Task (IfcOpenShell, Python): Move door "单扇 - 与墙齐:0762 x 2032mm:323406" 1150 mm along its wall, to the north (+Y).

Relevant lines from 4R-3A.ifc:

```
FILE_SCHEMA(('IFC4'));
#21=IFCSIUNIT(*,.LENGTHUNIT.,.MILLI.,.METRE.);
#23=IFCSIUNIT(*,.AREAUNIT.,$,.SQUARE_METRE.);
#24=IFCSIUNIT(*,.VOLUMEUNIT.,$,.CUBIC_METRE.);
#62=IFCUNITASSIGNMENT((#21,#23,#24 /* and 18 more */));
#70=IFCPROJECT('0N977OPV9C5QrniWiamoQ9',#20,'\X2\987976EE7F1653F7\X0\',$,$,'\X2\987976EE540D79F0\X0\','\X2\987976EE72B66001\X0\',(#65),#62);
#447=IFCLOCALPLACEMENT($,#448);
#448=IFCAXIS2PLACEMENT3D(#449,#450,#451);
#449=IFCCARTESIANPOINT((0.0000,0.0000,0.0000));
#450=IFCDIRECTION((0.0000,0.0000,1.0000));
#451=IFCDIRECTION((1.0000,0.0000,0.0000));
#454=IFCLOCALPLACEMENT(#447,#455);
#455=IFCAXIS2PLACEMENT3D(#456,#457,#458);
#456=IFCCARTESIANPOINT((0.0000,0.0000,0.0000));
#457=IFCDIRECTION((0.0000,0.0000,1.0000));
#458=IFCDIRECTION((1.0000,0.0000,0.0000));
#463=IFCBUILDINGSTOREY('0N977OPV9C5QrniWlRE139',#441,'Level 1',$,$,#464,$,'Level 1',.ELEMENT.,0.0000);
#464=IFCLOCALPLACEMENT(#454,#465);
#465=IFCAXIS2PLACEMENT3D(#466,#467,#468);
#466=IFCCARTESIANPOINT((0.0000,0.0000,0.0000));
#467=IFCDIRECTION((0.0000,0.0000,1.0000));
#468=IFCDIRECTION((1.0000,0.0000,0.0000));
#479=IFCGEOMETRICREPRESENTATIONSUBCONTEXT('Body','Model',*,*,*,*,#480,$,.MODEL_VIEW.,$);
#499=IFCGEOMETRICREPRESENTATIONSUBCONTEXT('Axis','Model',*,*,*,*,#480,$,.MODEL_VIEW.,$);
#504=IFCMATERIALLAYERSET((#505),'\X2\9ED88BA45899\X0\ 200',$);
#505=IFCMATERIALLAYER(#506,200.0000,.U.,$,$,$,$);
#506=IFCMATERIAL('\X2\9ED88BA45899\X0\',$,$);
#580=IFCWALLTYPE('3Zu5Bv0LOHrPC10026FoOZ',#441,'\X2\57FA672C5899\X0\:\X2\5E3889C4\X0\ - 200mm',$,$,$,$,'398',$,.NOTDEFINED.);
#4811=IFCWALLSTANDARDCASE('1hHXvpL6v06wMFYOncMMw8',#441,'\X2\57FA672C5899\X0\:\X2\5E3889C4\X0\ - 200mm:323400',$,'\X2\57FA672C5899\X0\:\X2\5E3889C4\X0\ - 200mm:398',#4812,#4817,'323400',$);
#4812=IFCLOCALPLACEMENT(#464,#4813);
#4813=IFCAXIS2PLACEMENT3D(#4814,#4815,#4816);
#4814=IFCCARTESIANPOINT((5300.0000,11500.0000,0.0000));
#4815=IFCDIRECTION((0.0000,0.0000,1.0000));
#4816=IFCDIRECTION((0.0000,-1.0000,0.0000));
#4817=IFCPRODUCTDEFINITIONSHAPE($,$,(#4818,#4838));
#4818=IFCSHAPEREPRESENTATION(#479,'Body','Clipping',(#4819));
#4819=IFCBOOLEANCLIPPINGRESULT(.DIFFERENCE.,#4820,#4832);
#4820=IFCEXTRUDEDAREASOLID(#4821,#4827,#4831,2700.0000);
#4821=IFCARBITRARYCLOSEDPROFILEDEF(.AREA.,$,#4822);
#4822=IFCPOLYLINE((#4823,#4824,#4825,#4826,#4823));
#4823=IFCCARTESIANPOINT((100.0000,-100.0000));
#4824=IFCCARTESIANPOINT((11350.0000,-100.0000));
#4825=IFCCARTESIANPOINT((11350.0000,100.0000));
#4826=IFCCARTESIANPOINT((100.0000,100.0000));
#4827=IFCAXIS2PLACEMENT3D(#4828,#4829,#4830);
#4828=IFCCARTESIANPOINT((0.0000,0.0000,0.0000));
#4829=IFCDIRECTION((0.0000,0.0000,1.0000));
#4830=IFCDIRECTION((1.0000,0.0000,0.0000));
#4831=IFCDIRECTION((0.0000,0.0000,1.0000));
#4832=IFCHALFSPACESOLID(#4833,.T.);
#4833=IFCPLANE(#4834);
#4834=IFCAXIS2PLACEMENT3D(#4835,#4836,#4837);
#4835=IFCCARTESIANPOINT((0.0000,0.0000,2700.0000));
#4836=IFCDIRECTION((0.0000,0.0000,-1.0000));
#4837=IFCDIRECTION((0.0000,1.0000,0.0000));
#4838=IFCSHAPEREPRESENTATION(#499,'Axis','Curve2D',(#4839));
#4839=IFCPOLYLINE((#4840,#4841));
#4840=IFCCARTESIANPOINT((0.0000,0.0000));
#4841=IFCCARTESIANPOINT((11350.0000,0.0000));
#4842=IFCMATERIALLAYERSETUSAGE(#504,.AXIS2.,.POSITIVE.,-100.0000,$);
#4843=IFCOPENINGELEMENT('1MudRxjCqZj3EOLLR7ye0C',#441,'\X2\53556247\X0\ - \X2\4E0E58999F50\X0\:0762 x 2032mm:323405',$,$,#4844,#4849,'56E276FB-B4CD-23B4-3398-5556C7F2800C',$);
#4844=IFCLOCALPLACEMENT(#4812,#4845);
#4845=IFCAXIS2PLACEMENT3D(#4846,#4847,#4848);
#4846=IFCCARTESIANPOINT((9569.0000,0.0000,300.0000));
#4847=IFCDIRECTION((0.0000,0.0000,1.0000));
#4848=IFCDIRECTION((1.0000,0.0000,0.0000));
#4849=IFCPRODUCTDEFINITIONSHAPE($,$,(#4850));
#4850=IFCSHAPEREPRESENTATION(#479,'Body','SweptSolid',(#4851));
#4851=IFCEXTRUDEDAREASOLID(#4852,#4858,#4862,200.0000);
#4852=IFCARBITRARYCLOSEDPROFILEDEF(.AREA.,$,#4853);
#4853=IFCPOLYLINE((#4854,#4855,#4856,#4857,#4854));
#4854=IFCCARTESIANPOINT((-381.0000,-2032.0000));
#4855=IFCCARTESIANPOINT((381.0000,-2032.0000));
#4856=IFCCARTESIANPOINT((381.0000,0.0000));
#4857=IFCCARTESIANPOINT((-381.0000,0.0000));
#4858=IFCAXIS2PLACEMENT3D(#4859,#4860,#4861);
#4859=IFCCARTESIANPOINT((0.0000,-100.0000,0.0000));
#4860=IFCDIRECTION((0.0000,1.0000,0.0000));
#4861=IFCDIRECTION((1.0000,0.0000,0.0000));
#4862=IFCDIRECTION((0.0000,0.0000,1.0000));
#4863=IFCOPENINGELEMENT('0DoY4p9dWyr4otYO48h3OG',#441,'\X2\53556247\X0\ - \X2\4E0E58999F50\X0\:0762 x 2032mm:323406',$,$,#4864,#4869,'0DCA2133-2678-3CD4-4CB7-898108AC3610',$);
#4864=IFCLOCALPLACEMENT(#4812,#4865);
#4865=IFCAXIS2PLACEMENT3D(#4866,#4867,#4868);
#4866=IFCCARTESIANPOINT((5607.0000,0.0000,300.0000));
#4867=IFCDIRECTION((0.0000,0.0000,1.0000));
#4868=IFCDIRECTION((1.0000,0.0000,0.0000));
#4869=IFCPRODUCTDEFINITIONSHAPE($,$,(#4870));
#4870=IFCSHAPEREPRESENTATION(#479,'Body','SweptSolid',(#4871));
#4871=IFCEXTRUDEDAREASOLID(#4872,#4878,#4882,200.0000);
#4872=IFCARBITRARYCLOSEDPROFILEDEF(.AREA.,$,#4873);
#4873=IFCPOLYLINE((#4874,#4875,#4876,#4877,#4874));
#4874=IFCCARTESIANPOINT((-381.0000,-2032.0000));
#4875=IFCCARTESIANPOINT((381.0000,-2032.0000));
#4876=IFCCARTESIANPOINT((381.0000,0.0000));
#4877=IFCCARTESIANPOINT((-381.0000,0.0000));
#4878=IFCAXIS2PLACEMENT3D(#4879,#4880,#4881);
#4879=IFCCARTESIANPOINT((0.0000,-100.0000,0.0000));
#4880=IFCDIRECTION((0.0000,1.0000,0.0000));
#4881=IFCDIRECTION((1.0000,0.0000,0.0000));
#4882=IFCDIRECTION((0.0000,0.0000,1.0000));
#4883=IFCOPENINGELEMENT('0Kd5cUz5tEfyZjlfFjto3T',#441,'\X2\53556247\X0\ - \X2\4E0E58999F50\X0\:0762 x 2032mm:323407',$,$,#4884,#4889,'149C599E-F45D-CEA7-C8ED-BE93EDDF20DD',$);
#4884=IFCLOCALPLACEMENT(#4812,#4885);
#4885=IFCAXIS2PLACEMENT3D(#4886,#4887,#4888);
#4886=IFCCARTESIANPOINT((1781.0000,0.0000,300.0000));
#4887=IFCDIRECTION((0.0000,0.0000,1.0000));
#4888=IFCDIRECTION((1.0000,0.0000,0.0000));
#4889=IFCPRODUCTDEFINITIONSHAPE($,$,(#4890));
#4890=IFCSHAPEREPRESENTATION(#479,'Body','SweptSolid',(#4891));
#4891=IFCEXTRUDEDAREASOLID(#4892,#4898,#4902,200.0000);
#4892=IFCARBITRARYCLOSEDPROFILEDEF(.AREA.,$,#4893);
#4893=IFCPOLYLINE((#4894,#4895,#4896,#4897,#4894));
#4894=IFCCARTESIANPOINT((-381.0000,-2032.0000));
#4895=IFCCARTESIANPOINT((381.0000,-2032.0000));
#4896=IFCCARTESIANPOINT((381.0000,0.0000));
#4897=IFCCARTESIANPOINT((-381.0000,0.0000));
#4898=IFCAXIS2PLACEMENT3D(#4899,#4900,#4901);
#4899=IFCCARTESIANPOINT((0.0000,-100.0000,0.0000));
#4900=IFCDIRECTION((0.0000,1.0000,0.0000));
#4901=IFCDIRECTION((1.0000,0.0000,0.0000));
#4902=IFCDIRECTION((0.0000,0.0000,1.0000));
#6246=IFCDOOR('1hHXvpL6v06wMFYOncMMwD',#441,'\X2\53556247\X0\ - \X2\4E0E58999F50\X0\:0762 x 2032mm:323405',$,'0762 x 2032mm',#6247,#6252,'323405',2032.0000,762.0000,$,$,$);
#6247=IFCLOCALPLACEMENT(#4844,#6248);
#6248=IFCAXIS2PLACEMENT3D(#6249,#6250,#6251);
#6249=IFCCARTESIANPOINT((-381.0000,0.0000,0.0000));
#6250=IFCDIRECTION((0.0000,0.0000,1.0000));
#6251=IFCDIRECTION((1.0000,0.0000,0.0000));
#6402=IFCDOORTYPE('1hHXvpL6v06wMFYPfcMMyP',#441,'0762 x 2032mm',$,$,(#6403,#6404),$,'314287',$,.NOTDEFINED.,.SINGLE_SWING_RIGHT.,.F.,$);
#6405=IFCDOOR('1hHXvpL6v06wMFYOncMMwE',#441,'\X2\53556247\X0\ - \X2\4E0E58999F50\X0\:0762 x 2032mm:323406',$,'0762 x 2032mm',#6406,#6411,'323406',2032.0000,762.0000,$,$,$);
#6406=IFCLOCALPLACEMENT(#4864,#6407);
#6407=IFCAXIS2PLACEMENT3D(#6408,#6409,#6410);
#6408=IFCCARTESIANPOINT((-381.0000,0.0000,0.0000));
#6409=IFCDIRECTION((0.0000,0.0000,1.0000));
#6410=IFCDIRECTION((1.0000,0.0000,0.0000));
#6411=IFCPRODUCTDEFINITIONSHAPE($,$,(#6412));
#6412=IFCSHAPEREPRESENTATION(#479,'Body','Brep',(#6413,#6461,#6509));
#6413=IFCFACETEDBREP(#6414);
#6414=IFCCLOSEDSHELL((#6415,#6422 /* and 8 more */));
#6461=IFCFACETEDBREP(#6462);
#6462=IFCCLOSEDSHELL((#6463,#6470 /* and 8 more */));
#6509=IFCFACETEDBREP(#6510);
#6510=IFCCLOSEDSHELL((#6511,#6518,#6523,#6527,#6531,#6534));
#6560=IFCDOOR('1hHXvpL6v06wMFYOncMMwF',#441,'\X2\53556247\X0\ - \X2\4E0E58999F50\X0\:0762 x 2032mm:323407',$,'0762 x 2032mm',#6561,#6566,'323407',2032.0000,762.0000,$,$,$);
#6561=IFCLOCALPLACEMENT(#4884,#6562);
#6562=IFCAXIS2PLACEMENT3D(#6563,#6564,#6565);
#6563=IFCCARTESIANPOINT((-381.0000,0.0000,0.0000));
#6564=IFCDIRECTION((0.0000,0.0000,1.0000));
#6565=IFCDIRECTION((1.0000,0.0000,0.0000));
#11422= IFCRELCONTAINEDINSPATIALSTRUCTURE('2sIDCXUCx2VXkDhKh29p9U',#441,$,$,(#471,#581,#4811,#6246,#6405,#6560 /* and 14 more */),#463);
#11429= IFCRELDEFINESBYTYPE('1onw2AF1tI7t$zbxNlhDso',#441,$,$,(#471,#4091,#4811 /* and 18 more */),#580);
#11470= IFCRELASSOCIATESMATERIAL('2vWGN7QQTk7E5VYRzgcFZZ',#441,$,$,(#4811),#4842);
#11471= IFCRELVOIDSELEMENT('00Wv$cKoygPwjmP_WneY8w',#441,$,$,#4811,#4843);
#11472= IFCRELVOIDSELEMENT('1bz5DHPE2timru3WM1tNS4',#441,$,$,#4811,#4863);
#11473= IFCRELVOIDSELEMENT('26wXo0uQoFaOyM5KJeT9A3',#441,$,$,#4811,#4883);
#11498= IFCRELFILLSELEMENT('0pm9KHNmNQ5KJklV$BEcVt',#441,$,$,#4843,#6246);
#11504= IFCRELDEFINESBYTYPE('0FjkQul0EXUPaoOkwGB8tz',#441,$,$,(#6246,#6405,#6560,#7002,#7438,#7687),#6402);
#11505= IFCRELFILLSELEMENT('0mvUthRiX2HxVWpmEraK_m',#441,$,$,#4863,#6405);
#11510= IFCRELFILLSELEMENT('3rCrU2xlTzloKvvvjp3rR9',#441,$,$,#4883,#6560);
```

```python
import ifcopenshell
import ifcopenshell.api.geometry
import ifcopenshell.util.placement

model = ifcopenshell.open("4R-3A.ifc")

door = model.by_guid("1hHXvpL6v06wMFYOncMMwE")
opening = door.FillsVoids[0].RelatingOpeningElement
wall = opening.VoidsElements[0].RelatingBuildingElement

wall_matrix = ifcopenshell.util.placement.get_local_placement(wall.ObjectPlacement)
shift = wall_matrix[:3, 0] * -1150.0
before = ifcopenshell.util.placement.get_local_placement(door.ObjectPlacement)[:3, 3].copy()

# The door is placed relative to its opening, so it follows when the opening moves.
matrix = ifcopenshell.util.placement.get_local_placement(opening.ObjectPlacement)
matrix[:3, 3] += shift
ifcopenshell.api.geometry.edit_object_placement(
    model, product=opening, matrix=matrix, is_si=False, should_transform_children=True
)

after = ifcopenshell.util.placement.get_local_placement(door.ObjectPlacement)[:3, 3]
print("door moved by", (after - before).round(3) + 0.0)

model.write("4R-3A_edited.ifc")
```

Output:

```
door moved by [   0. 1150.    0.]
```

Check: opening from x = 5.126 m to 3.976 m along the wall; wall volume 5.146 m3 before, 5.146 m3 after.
